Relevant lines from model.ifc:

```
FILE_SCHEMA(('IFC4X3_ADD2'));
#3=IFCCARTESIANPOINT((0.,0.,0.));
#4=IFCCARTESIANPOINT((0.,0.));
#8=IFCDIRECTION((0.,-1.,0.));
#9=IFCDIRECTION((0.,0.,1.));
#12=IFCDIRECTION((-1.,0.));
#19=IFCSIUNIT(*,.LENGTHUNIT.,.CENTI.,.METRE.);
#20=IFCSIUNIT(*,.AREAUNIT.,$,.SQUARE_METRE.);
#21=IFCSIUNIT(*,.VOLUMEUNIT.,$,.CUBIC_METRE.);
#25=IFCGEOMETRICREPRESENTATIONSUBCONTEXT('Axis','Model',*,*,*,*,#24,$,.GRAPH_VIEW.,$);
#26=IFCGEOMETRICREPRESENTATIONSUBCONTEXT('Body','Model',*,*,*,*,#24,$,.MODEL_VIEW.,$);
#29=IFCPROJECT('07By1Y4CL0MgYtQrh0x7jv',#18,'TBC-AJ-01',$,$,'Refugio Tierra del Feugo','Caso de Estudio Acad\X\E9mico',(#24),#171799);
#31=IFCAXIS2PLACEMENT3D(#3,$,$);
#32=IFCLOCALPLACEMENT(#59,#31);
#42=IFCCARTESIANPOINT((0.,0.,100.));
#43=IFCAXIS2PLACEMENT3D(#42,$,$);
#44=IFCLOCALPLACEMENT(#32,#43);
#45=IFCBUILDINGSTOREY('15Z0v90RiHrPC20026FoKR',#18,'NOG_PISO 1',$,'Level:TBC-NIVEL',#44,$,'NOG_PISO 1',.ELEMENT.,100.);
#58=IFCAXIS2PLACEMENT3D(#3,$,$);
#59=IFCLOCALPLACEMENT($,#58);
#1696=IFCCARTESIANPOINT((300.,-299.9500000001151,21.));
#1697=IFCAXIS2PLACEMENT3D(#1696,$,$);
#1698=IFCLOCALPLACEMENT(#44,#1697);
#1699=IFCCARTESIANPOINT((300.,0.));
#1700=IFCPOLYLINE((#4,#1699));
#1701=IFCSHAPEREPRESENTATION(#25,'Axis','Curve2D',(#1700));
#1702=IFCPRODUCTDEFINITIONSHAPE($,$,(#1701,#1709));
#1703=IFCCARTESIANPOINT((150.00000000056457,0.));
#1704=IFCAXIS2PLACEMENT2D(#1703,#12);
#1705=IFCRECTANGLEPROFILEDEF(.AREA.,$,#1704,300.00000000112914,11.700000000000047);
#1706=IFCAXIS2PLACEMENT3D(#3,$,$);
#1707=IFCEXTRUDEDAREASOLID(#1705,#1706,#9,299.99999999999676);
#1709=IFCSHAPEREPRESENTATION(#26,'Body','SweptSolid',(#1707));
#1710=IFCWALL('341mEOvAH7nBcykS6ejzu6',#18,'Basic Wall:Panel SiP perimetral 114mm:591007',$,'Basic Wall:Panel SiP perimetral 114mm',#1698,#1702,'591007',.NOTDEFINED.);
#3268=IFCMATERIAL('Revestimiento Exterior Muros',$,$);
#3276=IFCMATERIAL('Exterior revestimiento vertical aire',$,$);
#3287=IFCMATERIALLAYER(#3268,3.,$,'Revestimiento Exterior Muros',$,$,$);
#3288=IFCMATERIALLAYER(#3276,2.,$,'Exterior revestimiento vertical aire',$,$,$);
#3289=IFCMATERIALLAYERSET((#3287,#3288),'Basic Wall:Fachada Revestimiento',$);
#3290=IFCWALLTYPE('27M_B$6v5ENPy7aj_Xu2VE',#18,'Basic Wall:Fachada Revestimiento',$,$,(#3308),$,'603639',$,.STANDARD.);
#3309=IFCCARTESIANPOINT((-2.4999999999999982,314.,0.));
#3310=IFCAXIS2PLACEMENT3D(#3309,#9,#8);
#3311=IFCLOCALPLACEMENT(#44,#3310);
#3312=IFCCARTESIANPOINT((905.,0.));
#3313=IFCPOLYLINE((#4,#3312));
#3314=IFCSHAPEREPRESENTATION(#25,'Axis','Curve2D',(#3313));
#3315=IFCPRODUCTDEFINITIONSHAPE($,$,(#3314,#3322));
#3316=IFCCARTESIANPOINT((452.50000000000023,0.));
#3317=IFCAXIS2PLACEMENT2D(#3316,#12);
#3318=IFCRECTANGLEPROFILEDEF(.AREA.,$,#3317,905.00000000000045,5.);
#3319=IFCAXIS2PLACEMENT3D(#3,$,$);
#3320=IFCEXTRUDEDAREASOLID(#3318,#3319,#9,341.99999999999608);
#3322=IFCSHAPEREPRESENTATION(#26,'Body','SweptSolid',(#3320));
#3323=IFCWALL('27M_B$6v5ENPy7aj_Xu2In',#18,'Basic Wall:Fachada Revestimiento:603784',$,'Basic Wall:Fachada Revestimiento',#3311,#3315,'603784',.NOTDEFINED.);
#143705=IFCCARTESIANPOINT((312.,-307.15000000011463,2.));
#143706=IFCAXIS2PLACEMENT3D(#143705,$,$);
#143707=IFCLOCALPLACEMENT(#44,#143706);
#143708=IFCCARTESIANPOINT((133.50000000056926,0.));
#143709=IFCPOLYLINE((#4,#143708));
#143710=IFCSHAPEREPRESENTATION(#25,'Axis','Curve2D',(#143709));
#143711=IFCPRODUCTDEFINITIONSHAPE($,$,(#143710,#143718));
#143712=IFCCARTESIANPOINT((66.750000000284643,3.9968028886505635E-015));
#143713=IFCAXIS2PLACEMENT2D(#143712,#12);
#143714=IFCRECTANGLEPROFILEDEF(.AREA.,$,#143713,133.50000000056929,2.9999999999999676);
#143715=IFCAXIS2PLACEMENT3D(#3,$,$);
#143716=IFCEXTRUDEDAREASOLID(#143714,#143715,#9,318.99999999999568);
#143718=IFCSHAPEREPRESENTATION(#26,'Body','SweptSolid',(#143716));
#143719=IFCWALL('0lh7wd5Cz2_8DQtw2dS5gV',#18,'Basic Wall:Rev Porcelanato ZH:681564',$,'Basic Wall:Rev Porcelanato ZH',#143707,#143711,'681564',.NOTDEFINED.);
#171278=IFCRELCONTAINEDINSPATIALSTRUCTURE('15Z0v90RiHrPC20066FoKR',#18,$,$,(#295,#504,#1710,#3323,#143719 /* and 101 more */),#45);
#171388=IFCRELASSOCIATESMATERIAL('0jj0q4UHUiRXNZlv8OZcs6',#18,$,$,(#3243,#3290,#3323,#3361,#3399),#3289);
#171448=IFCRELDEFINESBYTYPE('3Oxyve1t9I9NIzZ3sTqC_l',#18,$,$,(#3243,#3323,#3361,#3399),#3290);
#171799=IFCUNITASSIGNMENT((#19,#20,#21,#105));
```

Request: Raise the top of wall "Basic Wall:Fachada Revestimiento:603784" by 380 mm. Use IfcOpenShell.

```python
import ifcopenshell
import ifcopenshell.geom
import ifcopenshell.util.representation
import ifcopenshell.util.shape
import ifcopenshell.util.unit

model = ifcopenshell.open("model.ifc")
unit_scale = ifcopenshell.util.unit.calculate_unit_scale(model)
settings = ifcopenshell.geom.settings()


def volume(element):
    """Net volume in cubic metres, openings subtracted."""
    shape = ifcopenshell.geom.create_shape(settings, element)
    return ifcopenshell.util.shape.get_volume(shape.geometry)


wall = model.by_id(3323)
before = volume(wall)

body = ifcopenshell.util.representation.get_representation(wall, "Model", "Body")
solid = body.Items[0]
old_height = solid.Depth
solid.Depth += 0.38 / unit_scale
after = volume(wall)

print(f"height {old_height:g} -> {solid.Depth:g}, volume {before:.3f} -> {after:.3f} m3")

model.write("model_rev.ifc")
```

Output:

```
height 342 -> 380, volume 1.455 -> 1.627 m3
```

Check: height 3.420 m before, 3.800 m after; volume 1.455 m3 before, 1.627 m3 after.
